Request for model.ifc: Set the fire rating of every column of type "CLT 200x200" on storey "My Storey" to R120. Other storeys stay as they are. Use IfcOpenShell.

First a look at what the model holds.

```python
import ifcopenshell
import ifcopenshell.util.element

model = ifcopenshell.open("model.ifc")
print(model.schema)
storey = next(s for s in model.by_type("IfcBuildingStorey") if s.Name == "My Storey")
columns = [e for e in ifcopenshell.util.element.get_decomposition(storey) if e.is_a("IfcColumn")]
seen = {}
for e in columns:
    element_type = ifcopenshell.util.element.get_type(e)
    key = (element_type.Name if element_type != e and element_type else None, ifcopenshell.util.element.get_pset(e, "Pset_ColumnCommon", "FireRating"))
    seen[key] = seen.get(key, 0) + 1
for (name, value), count in sorted(seen.items(), key=str):
    print(count, "x", name, "|", value)
```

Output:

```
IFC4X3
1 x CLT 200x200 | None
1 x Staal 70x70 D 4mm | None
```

```python
import ifcopenshell
import ifcopenshell.api.pset
import ifcopenshell.util.element

model = ifcopenshell.open("model.ifc")

storey = next(s for s in model.by_type("IfcBuildingStorey") if s.Name == "My Storey")
columns = [e for e in ifcopenshell.util.element.get_decomposition(storey) if e.is_a("IfcColumn")]

count = 0
for e in columns:
    element_type = ifcopenshell.util.element.get_type(e)
    if element_type in (None, e) or element_type.Name != "CLT 200x200":
        continue
    # add_pset returns the element's existing set when there is one.
    pset = ifcopenshell.api.pset.add_pset(model, product=e, name="Pset_ColumnCommon")
    ifcopenshell.api.pset.edit_pset(model, pset=pset, properties={"FireRating": "R120"})
    count += 1

print(count, "columns updated")

model.write("model_updated.ifc")
```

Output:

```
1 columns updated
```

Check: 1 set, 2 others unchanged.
